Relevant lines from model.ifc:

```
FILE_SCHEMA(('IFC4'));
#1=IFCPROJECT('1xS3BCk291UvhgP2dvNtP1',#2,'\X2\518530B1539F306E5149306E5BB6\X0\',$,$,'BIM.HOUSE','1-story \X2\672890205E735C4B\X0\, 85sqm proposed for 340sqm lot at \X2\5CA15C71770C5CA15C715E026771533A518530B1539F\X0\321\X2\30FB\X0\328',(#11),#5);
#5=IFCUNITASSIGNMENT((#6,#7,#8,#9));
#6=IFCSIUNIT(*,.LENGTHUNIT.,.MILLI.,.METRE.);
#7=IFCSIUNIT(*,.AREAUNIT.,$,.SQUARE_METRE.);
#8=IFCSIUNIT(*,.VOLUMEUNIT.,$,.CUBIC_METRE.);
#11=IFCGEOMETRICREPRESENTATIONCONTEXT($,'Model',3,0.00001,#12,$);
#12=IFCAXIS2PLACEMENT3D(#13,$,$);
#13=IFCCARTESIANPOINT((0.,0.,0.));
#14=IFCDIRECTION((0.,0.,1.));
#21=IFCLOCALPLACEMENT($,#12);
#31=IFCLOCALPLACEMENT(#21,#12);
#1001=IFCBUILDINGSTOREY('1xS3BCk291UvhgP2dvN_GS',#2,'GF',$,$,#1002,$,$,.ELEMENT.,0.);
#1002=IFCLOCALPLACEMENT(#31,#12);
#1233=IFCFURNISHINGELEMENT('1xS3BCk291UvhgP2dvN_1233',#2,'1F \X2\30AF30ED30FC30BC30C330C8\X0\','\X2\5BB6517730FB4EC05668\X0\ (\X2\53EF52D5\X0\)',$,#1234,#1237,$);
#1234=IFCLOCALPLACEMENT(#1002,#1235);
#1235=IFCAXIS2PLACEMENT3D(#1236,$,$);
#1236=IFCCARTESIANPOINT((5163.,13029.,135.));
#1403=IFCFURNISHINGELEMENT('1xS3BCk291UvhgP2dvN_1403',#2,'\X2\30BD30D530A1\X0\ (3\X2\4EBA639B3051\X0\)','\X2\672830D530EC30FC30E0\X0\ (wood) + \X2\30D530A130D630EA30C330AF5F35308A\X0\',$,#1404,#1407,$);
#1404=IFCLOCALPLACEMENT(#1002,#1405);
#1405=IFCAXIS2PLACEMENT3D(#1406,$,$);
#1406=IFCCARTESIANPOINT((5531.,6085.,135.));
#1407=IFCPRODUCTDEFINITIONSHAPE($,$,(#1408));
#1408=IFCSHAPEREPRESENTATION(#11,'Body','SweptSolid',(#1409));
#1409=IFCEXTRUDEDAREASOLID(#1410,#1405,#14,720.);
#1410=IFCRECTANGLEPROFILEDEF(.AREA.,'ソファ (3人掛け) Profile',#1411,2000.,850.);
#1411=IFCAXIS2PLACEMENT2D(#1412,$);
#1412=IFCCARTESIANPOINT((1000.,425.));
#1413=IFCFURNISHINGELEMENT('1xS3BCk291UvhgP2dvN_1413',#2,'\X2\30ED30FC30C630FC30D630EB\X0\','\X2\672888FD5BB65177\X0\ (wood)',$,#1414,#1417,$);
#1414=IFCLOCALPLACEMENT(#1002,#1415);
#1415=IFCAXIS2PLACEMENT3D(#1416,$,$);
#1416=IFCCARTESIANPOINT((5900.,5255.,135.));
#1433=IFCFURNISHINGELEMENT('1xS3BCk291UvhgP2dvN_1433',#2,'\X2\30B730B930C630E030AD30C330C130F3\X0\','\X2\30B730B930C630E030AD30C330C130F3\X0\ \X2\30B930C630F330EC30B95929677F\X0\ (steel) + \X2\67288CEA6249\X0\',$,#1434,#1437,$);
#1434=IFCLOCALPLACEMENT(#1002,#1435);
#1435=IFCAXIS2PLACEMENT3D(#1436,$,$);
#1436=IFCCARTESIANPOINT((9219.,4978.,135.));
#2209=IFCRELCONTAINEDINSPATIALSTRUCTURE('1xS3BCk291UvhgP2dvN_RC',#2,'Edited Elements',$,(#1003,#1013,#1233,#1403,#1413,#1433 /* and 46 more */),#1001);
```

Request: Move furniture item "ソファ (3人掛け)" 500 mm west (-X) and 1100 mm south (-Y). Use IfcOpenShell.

```python
import ifcopenshell
import ifcopenshell.api.geometry
import ifcopenshell.util.placement

model = ifcopenshell.open("model.ifc")

item = model.by_id(1403)
matrix = ifcopenshell.util.placement.get_local_placement(item.ObjectPlacement)
matrix[0, 3] -= 500.0
matrix[1, 3] -= 1100.0
ifcopenshell.api.geometry.edit_object_placement(model, product=item, matrix=matrix, is_si=False)

print(ifcopenshell.util.placement.get_local_placement(item.ObjectPlacement).round(3) + 0.0)

model.write("model_edited.ifc")
```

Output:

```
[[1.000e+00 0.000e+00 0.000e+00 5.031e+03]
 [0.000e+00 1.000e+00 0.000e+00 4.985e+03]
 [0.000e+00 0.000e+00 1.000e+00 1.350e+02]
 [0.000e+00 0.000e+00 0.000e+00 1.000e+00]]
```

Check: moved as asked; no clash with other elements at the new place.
